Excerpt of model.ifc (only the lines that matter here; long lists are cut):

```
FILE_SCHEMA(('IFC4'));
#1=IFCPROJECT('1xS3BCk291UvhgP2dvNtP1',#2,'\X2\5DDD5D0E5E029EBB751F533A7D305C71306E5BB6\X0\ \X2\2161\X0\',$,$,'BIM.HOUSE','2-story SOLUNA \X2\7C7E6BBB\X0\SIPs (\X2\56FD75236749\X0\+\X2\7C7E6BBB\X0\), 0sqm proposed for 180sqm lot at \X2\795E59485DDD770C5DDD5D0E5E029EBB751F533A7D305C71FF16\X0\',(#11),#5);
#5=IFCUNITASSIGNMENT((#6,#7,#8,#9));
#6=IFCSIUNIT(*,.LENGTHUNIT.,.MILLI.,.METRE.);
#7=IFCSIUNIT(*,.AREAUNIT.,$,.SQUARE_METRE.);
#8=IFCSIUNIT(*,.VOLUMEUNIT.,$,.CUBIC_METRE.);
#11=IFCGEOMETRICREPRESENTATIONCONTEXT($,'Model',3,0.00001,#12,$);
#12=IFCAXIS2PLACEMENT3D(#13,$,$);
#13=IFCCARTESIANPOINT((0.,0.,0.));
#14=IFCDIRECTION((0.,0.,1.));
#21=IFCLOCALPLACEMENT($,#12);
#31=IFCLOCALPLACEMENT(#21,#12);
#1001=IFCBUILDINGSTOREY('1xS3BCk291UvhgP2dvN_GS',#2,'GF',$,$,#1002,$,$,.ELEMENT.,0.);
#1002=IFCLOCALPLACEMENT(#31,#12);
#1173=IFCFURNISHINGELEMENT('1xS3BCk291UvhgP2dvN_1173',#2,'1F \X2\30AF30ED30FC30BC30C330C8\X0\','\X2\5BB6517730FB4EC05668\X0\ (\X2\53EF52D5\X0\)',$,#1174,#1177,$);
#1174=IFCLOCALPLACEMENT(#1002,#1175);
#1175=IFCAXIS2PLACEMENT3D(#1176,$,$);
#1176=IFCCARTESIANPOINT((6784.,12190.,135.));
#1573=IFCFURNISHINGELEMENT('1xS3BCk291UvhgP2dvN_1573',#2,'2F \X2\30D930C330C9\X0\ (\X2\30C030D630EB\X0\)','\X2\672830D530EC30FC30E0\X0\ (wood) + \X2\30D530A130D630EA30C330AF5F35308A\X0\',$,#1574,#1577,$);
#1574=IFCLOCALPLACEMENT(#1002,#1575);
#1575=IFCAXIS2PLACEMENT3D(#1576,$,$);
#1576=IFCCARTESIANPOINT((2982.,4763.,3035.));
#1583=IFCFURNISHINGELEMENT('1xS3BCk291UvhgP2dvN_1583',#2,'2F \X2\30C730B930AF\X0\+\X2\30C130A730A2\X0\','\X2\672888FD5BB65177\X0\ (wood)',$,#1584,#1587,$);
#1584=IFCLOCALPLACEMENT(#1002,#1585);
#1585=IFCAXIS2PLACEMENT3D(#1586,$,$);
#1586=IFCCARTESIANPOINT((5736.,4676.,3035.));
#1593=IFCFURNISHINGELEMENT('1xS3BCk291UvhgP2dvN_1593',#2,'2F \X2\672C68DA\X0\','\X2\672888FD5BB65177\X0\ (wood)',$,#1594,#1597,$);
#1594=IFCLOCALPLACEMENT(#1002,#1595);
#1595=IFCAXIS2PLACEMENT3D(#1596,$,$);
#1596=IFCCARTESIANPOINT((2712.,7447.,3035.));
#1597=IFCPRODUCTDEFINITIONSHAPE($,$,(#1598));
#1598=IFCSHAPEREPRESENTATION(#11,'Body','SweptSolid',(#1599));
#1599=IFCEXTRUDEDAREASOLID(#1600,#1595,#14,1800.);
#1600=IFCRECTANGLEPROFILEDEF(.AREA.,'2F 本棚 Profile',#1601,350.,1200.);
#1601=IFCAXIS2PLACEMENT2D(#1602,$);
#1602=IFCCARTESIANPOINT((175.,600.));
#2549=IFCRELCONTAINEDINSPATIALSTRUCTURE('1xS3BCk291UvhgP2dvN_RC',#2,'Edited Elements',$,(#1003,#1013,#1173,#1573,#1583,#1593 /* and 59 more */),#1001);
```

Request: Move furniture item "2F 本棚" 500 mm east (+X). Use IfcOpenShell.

```python
import ifcopenshell
import ifcopenshell.api.geometry
import ifcopenshell.util.placement

model = ifcopenshell.open("model.ifc")

item = model.by_guid("1xS3BCk291UvhgP2dvN_1593")
matrix = ifcopenshell.util.placement.get_local_placement(item.ObjectPlacement)
matrix[0, 3] += 500.0
ifcopenshell.api.geometry.edit_object_placement(model, product=item, matrix=matrix, is_si=False)

print(ifcopenshell.util.placement.get_local_placement(item.ObjectPlacement).round(3) + 0.0)

model.write("model_updated.ifc")
```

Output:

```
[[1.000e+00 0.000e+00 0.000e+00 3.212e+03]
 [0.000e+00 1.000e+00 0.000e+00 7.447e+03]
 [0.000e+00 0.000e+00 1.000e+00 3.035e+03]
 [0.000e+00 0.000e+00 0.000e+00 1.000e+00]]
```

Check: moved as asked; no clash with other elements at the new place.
